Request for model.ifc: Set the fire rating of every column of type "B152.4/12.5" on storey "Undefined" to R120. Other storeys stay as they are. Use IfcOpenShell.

First a look at what the model holds.

```python
import ifcopenshell
import ifcopenshell.util.element

model = ifcopenshell.open("model.ifc")
print(model.schema)
storey = next(s for s in model.by_type("IfcBuildingStorey") if s.Name == "Undefined")
columns = [e for e in ifcopenshell.util.element.get_decomposition(storey) if e.is_a("IfcColumn")]
seen = {}
for e in columns:
    element_type = ifcopenshell.util.element.get_type(e)
    key = (element_type.Name if element_type != e and element_type else None, ifcopenshell.util.element.get_pset(e, "Pset_ColumnCommon", "FireRating"))
    seen[key] = seen.get(key, 0) + 1
for (name, value), count in sorted(seen.items(), key=str):
    print(count, "x", name, "|", value)
```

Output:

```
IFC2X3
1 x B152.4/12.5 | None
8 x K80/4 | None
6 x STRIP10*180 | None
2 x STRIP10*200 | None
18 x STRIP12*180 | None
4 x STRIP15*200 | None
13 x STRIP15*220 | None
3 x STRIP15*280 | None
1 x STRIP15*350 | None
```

```python
import ifcopenshell
import ifcopenshell.api.pset
import ifcopenshell.util.element

model = ifcopenshell.open("model.ifc")

storey = next(s for s in model.by_type("IfcBuildingStorey") if s.Name == "Undefined")
columns = [e for e in ifcopenshell.util.element.get_decomposition(storey) if e.is_a("IfcColumn")]

count = 0
for e in columns:
    element_type = ifcopenshell.util.element.get_type(e)
    if element_type in (None, e) or element_type.Name != "B152.4/12.5":
        continue
    # add_pset returns the element's existing set when there is one.
    pset = ifcopenshell.api.pset.add_pset(model, product=e, name="Pset_ColumnCommon")
    ifcopenshell.api.pset.edit_pset(model, pset=pset, properties={"FireRating": "R120"})
    count += 1

print(count, "columns updated")

model.write("model_v2.ifc")
```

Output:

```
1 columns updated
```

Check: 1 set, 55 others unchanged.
